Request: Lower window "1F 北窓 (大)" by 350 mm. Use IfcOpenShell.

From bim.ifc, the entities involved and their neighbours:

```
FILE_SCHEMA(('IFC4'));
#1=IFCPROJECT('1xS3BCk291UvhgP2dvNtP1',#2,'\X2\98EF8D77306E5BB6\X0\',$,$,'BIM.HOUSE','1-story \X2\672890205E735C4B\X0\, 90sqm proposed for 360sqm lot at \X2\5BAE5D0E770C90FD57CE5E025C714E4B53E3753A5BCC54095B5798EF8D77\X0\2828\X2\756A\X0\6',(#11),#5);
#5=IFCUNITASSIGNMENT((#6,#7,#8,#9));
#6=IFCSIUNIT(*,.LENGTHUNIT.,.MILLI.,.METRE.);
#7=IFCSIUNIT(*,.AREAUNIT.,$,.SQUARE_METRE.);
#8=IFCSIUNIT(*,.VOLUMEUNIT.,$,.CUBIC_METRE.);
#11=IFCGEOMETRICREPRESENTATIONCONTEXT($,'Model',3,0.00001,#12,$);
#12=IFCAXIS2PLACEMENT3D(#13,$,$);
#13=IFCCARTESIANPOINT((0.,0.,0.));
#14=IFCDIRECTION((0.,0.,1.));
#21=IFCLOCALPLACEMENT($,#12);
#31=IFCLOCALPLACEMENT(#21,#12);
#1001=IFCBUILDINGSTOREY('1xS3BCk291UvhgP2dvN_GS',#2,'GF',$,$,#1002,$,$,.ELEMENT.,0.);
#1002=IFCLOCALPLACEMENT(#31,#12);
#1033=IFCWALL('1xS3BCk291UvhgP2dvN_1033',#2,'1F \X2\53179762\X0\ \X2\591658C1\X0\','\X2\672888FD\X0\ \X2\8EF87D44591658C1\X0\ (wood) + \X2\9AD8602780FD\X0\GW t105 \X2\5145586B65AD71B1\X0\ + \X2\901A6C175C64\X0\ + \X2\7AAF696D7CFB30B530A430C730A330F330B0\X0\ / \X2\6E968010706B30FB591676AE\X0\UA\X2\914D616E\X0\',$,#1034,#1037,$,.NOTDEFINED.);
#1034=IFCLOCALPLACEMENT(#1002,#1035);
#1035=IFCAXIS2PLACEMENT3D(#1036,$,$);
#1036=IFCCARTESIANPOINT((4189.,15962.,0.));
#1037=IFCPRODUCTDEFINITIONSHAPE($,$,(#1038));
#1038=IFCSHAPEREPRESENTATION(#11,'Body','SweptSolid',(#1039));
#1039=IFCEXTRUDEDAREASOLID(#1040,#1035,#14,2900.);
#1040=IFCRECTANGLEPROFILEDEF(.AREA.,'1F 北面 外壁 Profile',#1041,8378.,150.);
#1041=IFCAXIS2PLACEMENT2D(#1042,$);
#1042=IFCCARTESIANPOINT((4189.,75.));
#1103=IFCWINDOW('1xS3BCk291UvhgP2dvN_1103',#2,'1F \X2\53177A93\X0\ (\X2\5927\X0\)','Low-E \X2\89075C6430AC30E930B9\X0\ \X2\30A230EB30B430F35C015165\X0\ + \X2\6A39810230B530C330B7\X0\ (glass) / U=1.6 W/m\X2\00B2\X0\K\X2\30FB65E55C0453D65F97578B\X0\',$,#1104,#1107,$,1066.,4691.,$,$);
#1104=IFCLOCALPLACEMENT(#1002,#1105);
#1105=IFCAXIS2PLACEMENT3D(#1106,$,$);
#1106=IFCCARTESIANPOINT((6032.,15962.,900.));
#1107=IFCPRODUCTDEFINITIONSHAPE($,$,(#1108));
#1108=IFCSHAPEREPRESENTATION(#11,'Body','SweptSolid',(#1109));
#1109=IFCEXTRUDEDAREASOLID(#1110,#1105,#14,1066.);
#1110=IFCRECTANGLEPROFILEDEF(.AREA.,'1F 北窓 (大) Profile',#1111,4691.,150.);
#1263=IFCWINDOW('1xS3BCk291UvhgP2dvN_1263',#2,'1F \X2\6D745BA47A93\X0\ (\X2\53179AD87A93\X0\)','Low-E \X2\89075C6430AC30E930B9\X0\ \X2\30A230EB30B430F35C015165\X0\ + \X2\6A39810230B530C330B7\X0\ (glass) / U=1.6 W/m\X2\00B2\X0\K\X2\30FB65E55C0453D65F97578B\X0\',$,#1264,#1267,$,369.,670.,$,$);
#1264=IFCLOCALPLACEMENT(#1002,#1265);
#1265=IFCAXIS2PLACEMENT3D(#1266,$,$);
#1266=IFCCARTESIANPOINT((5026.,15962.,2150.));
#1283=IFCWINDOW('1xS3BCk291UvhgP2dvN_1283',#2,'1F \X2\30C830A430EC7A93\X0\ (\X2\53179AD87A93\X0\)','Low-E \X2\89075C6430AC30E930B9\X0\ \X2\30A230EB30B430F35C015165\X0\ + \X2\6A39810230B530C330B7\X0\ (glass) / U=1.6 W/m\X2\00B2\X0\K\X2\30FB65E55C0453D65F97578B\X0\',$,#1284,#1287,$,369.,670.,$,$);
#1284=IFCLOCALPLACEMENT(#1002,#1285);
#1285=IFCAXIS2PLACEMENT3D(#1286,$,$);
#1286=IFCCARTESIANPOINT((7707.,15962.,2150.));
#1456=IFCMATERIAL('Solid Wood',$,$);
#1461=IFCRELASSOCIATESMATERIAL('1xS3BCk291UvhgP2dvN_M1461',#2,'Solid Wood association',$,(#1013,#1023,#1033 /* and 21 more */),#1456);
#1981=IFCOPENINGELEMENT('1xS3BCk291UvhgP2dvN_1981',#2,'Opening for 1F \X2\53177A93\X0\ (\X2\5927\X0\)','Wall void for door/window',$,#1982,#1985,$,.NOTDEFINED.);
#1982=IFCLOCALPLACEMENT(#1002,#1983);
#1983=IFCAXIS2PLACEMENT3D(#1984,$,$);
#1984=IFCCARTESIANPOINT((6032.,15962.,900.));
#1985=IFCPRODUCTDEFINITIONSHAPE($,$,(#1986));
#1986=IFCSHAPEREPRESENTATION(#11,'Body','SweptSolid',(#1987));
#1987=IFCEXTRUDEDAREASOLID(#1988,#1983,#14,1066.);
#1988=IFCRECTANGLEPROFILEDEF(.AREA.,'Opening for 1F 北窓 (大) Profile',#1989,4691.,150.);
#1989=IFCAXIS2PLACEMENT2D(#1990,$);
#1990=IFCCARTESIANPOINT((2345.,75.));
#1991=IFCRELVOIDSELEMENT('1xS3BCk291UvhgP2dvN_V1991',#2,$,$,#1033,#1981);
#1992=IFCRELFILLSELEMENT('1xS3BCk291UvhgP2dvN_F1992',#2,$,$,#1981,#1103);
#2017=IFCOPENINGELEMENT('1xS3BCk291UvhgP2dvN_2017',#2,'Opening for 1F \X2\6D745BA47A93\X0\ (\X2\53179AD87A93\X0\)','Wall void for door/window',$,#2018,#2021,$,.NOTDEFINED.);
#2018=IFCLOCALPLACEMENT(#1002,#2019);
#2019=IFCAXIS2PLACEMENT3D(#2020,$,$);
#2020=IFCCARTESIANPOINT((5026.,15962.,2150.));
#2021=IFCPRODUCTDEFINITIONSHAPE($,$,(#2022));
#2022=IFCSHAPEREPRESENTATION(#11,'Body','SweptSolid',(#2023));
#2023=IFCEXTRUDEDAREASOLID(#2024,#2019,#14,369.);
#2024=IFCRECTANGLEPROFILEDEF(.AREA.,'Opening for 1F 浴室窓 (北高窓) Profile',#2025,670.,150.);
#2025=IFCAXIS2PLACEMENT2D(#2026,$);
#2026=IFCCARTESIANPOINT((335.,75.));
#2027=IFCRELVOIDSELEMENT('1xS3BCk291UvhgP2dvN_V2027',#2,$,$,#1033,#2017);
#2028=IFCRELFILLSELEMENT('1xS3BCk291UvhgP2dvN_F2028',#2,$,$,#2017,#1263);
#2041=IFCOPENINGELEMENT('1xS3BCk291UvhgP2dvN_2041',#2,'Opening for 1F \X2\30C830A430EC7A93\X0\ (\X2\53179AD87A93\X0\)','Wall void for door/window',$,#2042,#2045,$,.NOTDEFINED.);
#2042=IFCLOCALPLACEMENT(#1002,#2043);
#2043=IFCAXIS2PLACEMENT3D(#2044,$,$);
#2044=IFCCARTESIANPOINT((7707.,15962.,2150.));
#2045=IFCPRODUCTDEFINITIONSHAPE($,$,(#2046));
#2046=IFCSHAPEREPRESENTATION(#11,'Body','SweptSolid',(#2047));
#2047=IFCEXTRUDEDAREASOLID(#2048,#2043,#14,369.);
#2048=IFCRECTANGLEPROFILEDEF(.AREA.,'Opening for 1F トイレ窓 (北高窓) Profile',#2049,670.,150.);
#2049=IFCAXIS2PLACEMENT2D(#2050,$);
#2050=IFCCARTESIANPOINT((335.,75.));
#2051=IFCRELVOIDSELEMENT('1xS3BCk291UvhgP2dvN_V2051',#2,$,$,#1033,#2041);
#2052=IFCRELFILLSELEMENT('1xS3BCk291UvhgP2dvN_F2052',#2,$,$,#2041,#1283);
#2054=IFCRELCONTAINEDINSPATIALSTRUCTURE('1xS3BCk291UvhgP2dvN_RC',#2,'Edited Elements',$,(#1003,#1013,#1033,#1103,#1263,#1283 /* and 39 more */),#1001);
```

```python
import numpy as np
import ifcopenshell
import ifcopenshell.api.geometry
import ifcopenshell.util.placement
import ifcopenshell.util.unit

model = ifcopenshell.open("bim.ifc")
unit_scale = ifcopenshell.util.unit.calculate_unit_scale(model)

window = model.by_guid("1xS3BCk291UvhgP2dvN_1103")
opening = window.FillsVoids[0].RelatingOpeningElement
dz = -0.35 / unit_scale

shift = np.array([0.0, 0.0, dz])
# The window is not placed relative to its opening, so move both.
for product in (opening, window):
    matrix = ifcopenshell.util.placement.get_local_placement(product.ObjectPlacement)
    matrix[:3, 3] += shift
    ifcopenshell.api.geometry.edit_object_placement(model, product=product, matrix=matrix, is_si=False)

print(f"moved by {dz * unit_scale:+.3f} m")

model.write("bim-out.ifc")
```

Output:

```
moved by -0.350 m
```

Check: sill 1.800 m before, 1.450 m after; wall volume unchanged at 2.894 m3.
